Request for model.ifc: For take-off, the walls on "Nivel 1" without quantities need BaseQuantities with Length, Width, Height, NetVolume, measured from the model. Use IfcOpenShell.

First a look at what the model holds.

```python
import ifcopenshell
import ifcopenshell.util.element
import ifcopenshell.util.unit

model = ifcopenshell.open("model.ifc")
print(model.schema)
for unit_type in ("LENGTHUNIT", "AREAUNIT", "VOLUMEUNIT"):
    print(unit_type, ifcopenshell.util.unit.calculate_unit_scale(model, unit_type))
storey = next(s for s in model.by_type("IfcBuildingStorey") if s.Name == "Nivel 1")
walls = [e for e in ifcopenshell.util.element.get_decomposition(storey) if e.is_a("IfcWall")]
for e in sorted(walls, key=lambda e: e.id()):
    print(e.id(), e.is_a(), e.Name, list(ifcopenshell.util.element.get_psets(e, qtos_only=True)), sep=" | ")
```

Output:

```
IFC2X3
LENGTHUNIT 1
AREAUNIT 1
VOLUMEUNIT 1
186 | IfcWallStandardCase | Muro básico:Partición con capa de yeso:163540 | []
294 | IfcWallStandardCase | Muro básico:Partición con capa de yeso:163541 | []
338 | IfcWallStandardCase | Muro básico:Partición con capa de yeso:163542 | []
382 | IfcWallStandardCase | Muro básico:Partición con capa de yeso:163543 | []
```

```python
import ifcopenshell
import ifcopenshell.api.pset
import ifcopenshell.geom
import ifcopenshell.util.element
import ifcopenshell.util.shape
import ifcopenshell.util.unit

model = ifcopenshell.open("model.ifc")
unit_scale = ifcopenshell.util.unit.calculate_unit_scale(model)
volume_scale = ifcopenshell.util.unit.calculate_unit_scale(model, "VOLUMEUNIT")
settings = ifcopenshell.geom.settings()

storey = next(s for s in model.by_type("IfcBuildingStorey") if s.Name == "Nivel 1")
walls = [e for e in ifcopenshell.util.element.get_decomposition(storey) if e.is_a("IfcWall")]

for e in sorted(walls, key=lambda e: e.id()):
    if ifcopenshell.util.element.get_psets(e, qtos_only=True, should_inherit=False):
        continue
    # Geometry comes back in metres, in the element's own axes.
    shape = ifcopenshell.geom.create_shape(settings, e)
    values = {
        "Length": ifcopenshell.util.shape.get_x(shape.geometry) / unit_scale,
        "Width": ifcopenshell.util.shape.get_y(shape.geometry) / unit_scale,
        "Height": ifcopenshell.util.shape.get_z(shape.geometry) / unit_scale,
        "NetVolume": ifcopenshell.util.shape.get_volume(shape.geometry) / volume_scale,
    }
    qto = ifcopenshell.api.pset.add_qto(model, product=e, name="BaseQuantities")
    ifcopenshell.api.pset.edit_qto(model, qto=qto, properties=values)
    print(e.id(), {k: round(v, 3) for k, v in values.items()})

model.write("model_rev.ifc")
```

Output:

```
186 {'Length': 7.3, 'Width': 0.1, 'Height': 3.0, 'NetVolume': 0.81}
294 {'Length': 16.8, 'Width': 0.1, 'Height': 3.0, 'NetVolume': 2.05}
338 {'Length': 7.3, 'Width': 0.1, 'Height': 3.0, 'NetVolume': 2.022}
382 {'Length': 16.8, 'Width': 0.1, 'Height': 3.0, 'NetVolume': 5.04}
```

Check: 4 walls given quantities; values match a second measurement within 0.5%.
